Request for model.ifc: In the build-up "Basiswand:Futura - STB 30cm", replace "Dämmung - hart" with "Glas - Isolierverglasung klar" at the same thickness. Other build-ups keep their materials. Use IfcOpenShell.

First a look at what the model holds.

```python
import ifcopenshell
import ifcopenshell.util.element

model = ifcopenshell.open("model.ifc")
print(model.schema)
for layer_set in model.by_type("IfcMaterialLayerSet"):
    if layer_set.LayerSetName == "Basiswand:Futura - STB 30cm":
        for layer in layer_set.MaterialLayers:
            print(layer.id(), layer.Material and layer.Material.Name, layer.LayerThickness, sep=" | ")
        print(len(ifcopenshell.util.element.get_elements_by_material(model, layer_set)), "elements and types use it")
print(sorted(m.Name for m in model.by_type("IfcMaterial") if m.Name)[:60])
```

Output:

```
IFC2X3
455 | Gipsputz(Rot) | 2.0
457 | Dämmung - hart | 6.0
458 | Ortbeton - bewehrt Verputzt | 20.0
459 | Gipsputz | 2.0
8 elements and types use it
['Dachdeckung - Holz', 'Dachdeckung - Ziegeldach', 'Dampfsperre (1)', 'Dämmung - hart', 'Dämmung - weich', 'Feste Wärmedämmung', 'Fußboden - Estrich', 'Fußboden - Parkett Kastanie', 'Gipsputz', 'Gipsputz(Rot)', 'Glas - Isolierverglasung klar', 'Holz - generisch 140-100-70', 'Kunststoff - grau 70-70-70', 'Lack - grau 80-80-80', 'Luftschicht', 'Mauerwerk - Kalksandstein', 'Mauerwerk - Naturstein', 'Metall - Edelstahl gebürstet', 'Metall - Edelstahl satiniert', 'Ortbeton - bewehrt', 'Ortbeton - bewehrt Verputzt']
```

```python
import ifcopenshell
import ifcopenshell.api.material

model = ifcopenshell.open("model.ifc")

layer_set = next(s for s in model.by_type("IfcMaterialLayerSet") if s.LayerSetName == "Basiswand:Futura - STB 30cm")
layer = next(l for l in layer_set.MaterialLayers if l.Material and l.Material.Name == "Dämmung - hart")
material = next(m for m in model.by_type("IfcMaterial") if m.Name == "Glas - Isolierverglasung klar")

# Point this one layer at the other material; renaming the old one would change it everywhere.
ifcopenshell.api.material.edit_layer(model, layer=layer, attributes={}, material=material)

print([l.Material.Name if l.Material else None for l in layer_set.MaterialLayers])

model.write("model_updated.ifc")
```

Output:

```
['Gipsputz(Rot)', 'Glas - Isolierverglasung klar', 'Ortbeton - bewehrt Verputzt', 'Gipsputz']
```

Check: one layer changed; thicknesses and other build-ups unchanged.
